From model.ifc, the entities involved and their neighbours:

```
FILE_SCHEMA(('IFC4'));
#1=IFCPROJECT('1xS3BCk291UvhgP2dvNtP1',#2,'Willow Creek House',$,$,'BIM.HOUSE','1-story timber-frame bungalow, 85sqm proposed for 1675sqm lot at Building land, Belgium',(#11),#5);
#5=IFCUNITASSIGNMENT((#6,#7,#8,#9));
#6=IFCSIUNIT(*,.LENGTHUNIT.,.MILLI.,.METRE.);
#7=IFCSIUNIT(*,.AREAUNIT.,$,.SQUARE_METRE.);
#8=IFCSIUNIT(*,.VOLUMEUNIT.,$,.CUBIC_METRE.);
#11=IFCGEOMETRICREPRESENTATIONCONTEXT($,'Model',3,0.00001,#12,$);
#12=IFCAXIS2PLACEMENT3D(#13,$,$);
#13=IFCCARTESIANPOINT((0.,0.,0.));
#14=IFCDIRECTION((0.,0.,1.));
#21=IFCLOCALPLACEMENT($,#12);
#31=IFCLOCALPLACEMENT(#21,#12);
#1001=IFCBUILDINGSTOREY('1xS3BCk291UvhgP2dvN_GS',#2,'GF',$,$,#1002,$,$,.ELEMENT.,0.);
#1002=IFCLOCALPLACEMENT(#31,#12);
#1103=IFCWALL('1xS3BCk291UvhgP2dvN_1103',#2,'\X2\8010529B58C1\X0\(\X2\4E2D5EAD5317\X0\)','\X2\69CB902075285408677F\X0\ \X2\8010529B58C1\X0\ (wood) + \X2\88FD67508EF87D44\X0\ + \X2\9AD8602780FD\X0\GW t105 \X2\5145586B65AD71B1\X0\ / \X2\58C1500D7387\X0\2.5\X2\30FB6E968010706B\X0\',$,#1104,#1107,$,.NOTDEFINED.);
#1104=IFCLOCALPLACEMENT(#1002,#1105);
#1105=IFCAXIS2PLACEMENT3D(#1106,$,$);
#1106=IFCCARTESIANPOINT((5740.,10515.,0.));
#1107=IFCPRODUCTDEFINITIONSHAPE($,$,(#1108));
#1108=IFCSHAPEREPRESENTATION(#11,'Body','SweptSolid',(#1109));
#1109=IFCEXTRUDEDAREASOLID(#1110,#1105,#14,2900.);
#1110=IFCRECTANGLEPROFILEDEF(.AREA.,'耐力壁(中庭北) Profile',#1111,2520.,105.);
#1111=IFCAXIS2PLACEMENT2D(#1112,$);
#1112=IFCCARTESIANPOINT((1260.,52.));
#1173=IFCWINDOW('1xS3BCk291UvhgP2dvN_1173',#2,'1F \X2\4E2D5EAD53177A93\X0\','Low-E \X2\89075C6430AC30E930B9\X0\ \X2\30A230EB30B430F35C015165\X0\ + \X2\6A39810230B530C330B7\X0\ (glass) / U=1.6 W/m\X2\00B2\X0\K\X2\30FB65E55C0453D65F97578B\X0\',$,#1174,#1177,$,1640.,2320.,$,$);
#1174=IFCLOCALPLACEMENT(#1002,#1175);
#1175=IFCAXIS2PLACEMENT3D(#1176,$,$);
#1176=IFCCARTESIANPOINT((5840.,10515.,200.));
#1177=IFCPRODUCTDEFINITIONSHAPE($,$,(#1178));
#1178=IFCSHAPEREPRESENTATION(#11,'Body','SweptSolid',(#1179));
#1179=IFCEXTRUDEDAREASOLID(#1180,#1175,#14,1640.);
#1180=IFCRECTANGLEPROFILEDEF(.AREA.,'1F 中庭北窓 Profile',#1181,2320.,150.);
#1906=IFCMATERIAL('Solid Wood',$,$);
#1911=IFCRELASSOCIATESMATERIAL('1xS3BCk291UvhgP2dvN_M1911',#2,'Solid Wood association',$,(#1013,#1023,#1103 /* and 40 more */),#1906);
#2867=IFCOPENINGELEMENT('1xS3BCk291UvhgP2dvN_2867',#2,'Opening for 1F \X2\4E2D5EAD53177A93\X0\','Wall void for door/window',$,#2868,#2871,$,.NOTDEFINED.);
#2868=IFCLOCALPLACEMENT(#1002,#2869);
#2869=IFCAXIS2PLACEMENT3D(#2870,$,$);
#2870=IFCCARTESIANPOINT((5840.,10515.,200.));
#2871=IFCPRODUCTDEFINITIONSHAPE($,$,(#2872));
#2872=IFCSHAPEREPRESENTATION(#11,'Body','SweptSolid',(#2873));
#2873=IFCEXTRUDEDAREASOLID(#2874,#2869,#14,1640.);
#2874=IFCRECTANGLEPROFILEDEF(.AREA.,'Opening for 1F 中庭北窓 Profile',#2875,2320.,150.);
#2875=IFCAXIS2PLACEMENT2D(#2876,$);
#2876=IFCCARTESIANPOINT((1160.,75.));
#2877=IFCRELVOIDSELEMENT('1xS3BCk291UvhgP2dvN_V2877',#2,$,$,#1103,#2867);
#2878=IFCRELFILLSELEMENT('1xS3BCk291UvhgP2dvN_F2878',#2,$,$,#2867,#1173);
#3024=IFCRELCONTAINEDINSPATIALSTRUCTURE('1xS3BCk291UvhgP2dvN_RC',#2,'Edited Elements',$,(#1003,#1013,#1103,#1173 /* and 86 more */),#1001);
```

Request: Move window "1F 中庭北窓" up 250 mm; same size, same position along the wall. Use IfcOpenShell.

```python
import numpy as np
import ifcopenshell
import ifcopenshell.api.geometry
import ifcopenshell.util.placement
import ifcopenshell.util.unit

model = ifcopenshell.open("model.ifc")
unit_scale = ifcopenshell.util.unit.calculate_unit_scale(model)

window = model.by_id(1173)
opening = window.FillsVoids[0].RelatingOpeningElement
dz = 250.0

shift = np.array([0.0, 0.0, dz])
# The window is not placed relative to its opening, so move both.
for product in (opening, window):
    matrix = ifcopenshell.util.placement.get_local_placement(product.ObjectPlacement)
    matrix[:3, 3] += shift
    ifcopenshell.api.geometry.edit_object_placement(model, product=product, matrix=matrix, is_si=False)

print(f"moved by {dz * unit_scale:+.3f} m")

model.write("model_updated.ifc")
```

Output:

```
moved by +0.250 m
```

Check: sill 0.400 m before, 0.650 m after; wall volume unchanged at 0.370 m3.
